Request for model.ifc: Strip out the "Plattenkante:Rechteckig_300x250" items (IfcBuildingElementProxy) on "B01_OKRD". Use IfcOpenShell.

First a look at what the model holds.

```python
import ifcopenshell
import ifcopenshell.util.element

model = ifcopenshell.open("model.ifc")
print(model.schema)
storey = next(s for s in model.by_type("IfcBuildingStorey") if s.Name == "B01_OKRD")
proxies = [e for e in ifcopenshell.util.element.get_decomposition(storey) if e.is_a("IfcBuildingElementProxy")]
seen = {}
for e in proxies:
    element_type = ifcopenshell.util.element.get_type(e)
    name = element_type.Name if element_type not in (None, e) else None
    seen[name] = seen.get(name, 0) + 1
for name, count in sorted(seen.items(), key=str):
    print(count, "x", name)
```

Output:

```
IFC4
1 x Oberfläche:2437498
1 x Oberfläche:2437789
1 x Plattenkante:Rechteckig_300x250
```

```python
import ifcopenshell
import ifcopenshell.api.root
import ifcopenshell.util.element

model = ifcopenshell.open("model.ifc")

storey = next(s for s in model.by_type("IfcBuildingStorey") if s.Name == "B01_OKRD")
proxies = [e for e in ifcopenshell.util.element.get_decomposition(storey) if e.is_a("IfcBuildingElementProxy")]
targets = [e for e in proxies if (t := ifcopenshell.util.element.get_type(e)) not in (None, e) and t.Name == "Plattenkante:Rechteckig_300x250"]

for e in targets:
    ifcopenshell.api.root.remove_product(model, product=e)
print(len(targets), "removed")

model.write("model_v2.ifc")
```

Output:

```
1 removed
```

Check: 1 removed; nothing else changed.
